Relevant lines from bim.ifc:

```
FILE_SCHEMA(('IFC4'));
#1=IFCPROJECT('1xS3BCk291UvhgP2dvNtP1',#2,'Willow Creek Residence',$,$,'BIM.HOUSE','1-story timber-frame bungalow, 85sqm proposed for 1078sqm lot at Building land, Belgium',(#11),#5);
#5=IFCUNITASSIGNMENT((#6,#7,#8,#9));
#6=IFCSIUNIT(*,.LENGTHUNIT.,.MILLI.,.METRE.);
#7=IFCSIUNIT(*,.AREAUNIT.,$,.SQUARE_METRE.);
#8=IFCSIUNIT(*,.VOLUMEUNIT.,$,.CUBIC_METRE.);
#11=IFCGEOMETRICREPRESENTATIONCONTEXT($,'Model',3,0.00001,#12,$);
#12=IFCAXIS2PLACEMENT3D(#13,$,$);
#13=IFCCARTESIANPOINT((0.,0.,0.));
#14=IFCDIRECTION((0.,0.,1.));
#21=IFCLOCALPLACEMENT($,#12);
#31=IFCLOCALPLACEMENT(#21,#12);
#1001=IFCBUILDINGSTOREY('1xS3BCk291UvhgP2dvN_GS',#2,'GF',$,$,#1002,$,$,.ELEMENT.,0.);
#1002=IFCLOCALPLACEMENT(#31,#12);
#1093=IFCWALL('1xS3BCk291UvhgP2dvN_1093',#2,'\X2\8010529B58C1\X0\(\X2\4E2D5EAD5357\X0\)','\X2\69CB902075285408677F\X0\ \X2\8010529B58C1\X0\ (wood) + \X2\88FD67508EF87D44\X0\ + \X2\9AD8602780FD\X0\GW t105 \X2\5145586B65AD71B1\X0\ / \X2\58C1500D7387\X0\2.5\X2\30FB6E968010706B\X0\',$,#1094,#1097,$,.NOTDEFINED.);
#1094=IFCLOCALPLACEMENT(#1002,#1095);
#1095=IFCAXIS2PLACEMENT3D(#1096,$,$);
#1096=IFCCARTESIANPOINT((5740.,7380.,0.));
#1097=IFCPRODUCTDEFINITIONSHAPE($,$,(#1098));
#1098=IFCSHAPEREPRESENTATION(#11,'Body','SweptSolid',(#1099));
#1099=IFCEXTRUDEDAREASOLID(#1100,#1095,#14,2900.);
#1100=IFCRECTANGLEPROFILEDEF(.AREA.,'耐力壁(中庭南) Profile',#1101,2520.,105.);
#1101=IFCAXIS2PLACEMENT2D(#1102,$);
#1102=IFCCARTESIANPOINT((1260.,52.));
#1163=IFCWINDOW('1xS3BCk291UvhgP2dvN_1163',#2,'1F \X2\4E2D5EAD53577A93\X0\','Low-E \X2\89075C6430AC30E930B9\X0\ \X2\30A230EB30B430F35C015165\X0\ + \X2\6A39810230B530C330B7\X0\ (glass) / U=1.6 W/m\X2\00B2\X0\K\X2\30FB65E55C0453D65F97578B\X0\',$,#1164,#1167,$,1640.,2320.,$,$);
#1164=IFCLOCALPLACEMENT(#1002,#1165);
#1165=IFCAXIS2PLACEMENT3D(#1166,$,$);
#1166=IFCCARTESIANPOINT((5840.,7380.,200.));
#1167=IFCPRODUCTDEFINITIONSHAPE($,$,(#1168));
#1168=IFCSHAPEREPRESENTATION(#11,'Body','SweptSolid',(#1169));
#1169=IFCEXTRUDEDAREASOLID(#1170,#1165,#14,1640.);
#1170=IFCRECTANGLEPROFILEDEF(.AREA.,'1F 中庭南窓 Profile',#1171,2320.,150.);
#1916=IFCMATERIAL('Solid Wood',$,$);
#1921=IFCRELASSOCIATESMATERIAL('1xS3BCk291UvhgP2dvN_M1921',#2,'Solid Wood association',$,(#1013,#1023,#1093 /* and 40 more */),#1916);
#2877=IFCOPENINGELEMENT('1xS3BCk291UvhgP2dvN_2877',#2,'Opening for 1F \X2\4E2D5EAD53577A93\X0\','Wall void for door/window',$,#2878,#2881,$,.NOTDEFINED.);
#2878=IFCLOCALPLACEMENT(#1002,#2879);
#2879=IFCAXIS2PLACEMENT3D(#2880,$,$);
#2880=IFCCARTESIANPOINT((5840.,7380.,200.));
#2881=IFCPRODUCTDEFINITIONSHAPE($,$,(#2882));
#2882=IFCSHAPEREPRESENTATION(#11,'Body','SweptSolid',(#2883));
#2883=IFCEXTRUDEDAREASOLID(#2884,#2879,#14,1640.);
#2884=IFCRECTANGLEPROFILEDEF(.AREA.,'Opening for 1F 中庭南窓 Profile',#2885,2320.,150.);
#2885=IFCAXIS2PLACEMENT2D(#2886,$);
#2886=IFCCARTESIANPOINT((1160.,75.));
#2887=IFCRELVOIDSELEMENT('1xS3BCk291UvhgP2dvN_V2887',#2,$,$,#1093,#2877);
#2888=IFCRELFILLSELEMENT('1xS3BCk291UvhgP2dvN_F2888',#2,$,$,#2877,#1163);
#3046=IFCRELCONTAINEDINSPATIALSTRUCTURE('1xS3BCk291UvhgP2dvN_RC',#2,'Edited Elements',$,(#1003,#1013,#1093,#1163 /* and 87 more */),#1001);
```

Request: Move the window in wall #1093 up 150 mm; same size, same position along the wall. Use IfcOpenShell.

```python
import numpy as np
import ifcopenshell
import ifcopenshell.api.geometry
import ifcopenshell.util.placement
import ifcopenshell.util.unit

model = ifcopenshell.open("bim.ifc")
unit_scale = ifcopenshell.util.unit.calculate_unit_scale(model)

window = model.by_id(1163)
opening = window.FillsVoids[0].RelatingOpeningElement
dz = 150.0

shift = np.array([0.0, 0.0, dz])
# The window is not placed relative to its opening, so move both.
for product in (opening, window):
    matrix = ifcopenshell.util.placement.get_local_placement(product.ObjectPlacement)
    matrix[:3, 3] += shift
    ifcopenshell.api.geometry.edit_object_placement(model, product=product, matrix=matrix, is_si=False)

print(f"moved by {dz * unit_scale:+.3f} m")

model.write("bim_updated.ifc")
```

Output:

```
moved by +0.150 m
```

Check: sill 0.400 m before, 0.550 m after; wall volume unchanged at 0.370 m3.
